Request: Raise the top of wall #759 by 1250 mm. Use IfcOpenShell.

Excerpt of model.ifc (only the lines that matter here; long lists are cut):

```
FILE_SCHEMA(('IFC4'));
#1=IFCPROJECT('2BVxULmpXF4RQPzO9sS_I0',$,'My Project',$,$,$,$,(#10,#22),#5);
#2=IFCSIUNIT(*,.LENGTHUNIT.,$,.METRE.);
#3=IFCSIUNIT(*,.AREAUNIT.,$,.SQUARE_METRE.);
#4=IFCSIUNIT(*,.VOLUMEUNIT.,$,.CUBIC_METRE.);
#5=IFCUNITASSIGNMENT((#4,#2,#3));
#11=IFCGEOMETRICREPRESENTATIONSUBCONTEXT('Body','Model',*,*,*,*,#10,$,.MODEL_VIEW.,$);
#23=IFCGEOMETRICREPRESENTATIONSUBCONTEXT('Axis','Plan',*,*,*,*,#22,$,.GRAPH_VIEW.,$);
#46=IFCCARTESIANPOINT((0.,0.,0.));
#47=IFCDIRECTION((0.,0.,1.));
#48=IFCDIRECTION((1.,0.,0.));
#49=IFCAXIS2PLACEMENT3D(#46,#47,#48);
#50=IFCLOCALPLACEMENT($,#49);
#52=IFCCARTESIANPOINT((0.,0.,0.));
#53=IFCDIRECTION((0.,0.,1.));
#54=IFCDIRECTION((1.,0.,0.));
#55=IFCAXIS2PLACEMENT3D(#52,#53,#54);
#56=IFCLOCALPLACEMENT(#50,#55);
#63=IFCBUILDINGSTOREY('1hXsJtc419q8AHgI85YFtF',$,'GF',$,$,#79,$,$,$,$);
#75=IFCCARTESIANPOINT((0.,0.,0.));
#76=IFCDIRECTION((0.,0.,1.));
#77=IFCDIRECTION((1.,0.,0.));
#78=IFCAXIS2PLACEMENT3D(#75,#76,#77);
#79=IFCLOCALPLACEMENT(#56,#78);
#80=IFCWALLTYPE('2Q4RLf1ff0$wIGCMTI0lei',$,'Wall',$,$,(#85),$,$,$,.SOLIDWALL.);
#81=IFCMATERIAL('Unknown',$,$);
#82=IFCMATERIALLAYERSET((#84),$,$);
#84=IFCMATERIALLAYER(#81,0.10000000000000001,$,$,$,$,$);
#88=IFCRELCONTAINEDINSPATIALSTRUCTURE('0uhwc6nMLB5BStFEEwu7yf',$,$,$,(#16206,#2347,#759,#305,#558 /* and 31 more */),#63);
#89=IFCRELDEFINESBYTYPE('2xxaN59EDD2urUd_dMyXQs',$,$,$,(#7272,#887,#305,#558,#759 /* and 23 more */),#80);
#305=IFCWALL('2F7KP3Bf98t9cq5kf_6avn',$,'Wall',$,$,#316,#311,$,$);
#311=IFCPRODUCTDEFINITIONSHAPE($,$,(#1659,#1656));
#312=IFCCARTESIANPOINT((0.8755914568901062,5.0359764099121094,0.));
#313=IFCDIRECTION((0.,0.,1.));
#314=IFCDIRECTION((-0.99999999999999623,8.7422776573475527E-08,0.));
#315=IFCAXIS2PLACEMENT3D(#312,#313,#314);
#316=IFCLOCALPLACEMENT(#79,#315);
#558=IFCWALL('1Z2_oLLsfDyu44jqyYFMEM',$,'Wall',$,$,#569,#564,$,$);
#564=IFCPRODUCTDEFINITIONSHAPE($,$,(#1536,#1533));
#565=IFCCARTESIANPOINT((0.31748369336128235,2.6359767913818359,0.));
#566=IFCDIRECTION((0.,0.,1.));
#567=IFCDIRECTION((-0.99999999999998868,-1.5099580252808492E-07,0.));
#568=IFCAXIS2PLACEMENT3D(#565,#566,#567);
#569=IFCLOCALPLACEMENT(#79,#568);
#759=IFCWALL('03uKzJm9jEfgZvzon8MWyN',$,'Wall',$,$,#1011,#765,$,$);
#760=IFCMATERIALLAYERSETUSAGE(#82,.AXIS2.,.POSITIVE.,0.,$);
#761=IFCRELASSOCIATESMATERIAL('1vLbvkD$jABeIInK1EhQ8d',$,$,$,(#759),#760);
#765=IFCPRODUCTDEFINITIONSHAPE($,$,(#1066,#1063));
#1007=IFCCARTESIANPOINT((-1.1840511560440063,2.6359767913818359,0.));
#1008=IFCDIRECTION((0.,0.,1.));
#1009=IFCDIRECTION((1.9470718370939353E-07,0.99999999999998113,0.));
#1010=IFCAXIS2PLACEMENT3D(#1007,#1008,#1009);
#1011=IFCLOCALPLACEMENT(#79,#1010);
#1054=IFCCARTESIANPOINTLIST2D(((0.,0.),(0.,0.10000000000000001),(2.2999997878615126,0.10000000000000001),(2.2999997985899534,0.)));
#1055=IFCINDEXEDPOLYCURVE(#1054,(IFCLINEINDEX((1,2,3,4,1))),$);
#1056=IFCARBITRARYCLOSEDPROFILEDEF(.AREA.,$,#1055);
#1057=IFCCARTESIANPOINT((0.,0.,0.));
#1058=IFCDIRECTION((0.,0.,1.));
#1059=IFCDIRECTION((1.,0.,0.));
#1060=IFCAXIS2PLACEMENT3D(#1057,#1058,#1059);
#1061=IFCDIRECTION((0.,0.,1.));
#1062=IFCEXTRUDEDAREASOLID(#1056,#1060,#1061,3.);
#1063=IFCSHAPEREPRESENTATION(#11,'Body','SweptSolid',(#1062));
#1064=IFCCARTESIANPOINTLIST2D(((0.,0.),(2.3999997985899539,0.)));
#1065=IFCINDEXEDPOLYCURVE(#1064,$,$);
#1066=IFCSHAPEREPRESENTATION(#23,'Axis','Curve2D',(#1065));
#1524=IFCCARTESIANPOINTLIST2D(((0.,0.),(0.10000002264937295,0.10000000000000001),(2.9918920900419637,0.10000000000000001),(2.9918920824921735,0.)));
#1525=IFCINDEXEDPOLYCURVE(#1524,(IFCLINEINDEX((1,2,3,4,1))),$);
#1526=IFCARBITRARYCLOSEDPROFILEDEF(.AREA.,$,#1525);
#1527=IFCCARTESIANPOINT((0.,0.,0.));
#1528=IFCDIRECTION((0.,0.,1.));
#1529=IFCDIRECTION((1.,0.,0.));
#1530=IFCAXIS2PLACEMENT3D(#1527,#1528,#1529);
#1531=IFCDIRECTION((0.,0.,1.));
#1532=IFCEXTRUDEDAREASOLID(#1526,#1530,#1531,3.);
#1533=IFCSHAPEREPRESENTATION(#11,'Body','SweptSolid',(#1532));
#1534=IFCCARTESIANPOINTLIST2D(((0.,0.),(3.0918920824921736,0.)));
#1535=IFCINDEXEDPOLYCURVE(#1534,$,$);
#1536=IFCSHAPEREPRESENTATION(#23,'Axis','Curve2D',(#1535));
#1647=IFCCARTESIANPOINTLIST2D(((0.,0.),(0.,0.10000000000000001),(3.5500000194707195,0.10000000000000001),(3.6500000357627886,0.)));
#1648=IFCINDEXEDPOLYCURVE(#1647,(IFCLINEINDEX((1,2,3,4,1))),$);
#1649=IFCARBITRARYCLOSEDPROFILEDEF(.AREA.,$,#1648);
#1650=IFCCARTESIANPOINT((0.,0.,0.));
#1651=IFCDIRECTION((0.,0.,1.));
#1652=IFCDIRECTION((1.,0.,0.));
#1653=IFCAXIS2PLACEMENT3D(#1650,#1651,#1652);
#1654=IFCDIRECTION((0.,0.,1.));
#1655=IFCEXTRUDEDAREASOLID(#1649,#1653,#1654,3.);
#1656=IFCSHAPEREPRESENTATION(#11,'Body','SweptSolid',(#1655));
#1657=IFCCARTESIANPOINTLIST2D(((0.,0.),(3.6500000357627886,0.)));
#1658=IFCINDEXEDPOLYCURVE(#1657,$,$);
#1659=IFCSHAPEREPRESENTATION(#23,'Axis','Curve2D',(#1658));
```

```python
import ifcopenshell
import ifcopenshell.geom
import ifcopenshell.util.representation
import ifcopenshell.util.shape
import ifcopenshell.util.unit

model = ifcopenshell.open("model.ifc")
unit_scale = ifcopenshell.util.unit.calculate_unit_scale(model)
settings = ifcopenshell.geom.settings()


def volume(element):
    """Net volume in cubic metres, openings subtracted."""
    shape = ifcopenshell.geom.create_shape(settings, element)
    return ifcopenshell.util.shape.get_volume(shape.geometry)


wall = model.by_id(759)
before = volume(wall)

body = ifcopenshell.util.representation.get_representation(wall, "Model", "Body")
solid = body.Items[0]
old_height = solid.Depth
solid.Depth += 1.25 / unit_scale
after = volume(wall)

print(f"height {old_height:g} -> {solid.Depth:g}, volume {before:.3f} -> {after:.3f} m3")

model.write("model_rev.ifc")
```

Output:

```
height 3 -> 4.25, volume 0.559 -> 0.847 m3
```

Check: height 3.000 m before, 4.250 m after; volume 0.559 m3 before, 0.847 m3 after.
